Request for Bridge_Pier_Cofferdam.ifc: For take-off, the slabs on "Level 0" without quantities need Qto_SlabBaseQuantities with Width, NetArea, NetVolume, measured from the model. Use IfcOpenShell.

First a look at what the model holds.

```python
import ifcopenshell
import ifcopenshell.util.element
import ifcopenshell.util.unit

model = ifcopenshell.open("Bridge_Pier_Cofferdam.ifc")
print(model.schema)
for unit_type in ("LENGTHUNIT", "AREAUNIT", "VOLUMEUNIT"):
    print(unit_type, ifcopenshell.util.unit.calculate_unit_scale(model, unit_type))
storey = next(s for s in model.by_type("IfcBuildingStorey") if s.Name == "Level 0")
slabs = [e for e in ifcopenshell.util.element.get_decomposition(storey) if e.is_a("IfcSlab")]
for e in sorted(slabs, key=lambda e: e.id()):
    print(e.id(), e.is_a(), e.Name, list(ifcopenshell.util.element.get_psets(e, qtos_only=True)), sep=" | ")
```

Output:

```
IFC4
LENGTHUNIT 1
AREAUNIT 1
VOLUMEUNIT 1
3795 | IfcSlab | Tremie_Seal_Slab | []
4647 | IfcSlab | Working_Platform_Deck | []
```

```python
import ifcopenshell
import ifcopenshell.api.pset
import ifcopenshell.geom
import ifcopenshell.util.element
import ifcopenshell.util.shape
import ifcopenshell.util.unit

model = ifcopenshell.open("Bridge_Pier_Cofferdam.ifc")
unit_scale = ifcopenshell.util.unit.calculate_unit_scale(model)
area_scale = ifcopenshell.util.unit.calculate_unit_scale(model, "AREAUNIT")
volume_scale = ifcopenshell.util.unit.calculate_unit_scale(model, "VOLUMEUNIT")
settings = ifcopenshell.geom.settings()

storey = next(s for s in model.by_type("IfcBuildingStorey") if s.Name == "Level 0")
slabs = [e for e in ifcopenshell.util.element.get_decomposition(storey) if e.is_a("IfcSlab")]

for e in sorted(slabs, key=lambda e: e.id()):
    if ifcopenshell.util.element.get_psets(e, qtos_only=True, should_inherit=False):
        continue
    # Geometry comes back in metres, in the element's own axes.
    shape = ifcopenshell.geom.create_shape(settings, e)
    values = {
        "Width": ifcopenshell.util.shape.get_z(shape.geometry) / unit_scale,
        "NetArea": ifcopenshell.util.shape.get_footprint_area(shape.geometry) / area_scale,
        "NetVolume": ifcopenshell.util.shape.get_volume(shape.geometry) / volume_scale,
    }
    qto = ifcopenshell.api.pset.add_qto(model, product=e, name="Qto_SlabBaseQuantities")
    ifcopenshell.api.pset.edit_qto(model, qto=qto, properties=values)
    print(e.id(), {k: round(v, 3) for k, v in values.items()})

model.write("Bridge_Pier_Cofferdam-out.ifc")
```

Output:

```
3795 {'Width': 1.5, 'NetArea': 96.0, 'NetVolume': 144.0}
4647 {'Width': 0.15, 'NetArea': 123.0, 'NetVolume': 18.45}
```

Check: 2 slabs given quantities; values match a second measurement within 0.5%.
